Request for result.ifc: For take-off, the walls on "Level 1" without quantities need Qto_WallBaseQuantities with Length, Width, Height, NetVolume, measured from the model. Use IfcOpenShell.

First a look at what the model holds.

```python
import ifcopenshell
import ifcopenshell.util.element
import ifcopenshell.util.unit

model = ifcopenshell.open("result.ifc")
print(model.schema)
for unit_type in ("LENGTHUNIT", "AREAUNIT", "VOLUMEUNIT"):
    print(unit_type, ifcopenshell.util.unit.calculate_unit_scale(model, unit_type))
storey = next(s for s in model.by_type("IfcBuildingStorey") if s.Name == "Level 1")
walls = [e for e in ifcopenshell.util.element.get_decomposition(storey) if e.is_a("IfcWall")]
for e in sorted(walls, key=lambda e: e.id()):
    print(e.id(), e.is_a(), e.Name, list(ifcopenshell.util.element.get_psets(e, qtos_only=True)), sep=" | ")
```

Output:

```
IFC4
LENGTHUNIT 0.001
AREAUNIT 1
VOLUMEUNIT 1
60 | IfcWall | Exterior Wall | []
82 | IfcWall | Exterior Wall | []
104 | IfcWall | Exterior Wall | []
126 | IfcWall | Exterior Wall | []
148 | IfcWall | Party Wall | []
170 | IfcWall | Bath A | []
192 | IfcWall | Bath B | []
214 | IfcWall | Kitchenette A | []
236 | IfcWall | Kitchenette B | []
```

```python
import ifcopenshell
import ifcopenshell.api.pset
import ifcopenshell.geom
import ifcopenshell.util.element
import ifcopenshell.util.shape
import ifcopenshell.util.unit

model = ifcopenshell.open("result.ifc")
unit_scale = ifcopenshell.util.unit.calculate_unit_scale(model)
volume_scale = ifcopenshell.util.unit.calculate_unit_scale(model, "VOLUMEUNIT")
settings = ifcopenshell.geom.settings()

storey = next(s for s in model.by_type("IfcBuildingStorey") if s.Name == "Level 1")
walls = [e for e in ifcopenshell.util.element.get_decomposition(storey) if e.is_a("IfcWall")]

for e in sorted(walls, key=lambda e: e.id()):
    if ifcopenshell.util.element.get_psets(e, qtos_only=True, should_inherit=False):
        continue
    # Geometry comes back in metres, in the element's own axes.
    shape = ifcopenshell.geom.create_shape(settings, e)
    values = {
        "Length": ifcopenshell.util.shape.get_x(shape.geometry) / unit_scale,
        "Width": ifcopenshell.util.shape.get_y(shape.geometry) / unit_scale,
        "Height": ifcopenshell.util.shape.get_z(shape.geometry) / unit_scale,
        "NetVolume": ifcopenshell.util.shape.get_volume(shape.geometry) / volume_scale,
    }
    qto = ifcopenshell.api.pset.add_qto(model, product=e, name="Qto_WallBaseQuantities")
    ifcopenshell.api.pset.edit_qto(model, qto=qto, properties=values)
    print(e.id(), {k: round(v, 3) for k, v in values.items()})

model.write("result-out.ifc")
```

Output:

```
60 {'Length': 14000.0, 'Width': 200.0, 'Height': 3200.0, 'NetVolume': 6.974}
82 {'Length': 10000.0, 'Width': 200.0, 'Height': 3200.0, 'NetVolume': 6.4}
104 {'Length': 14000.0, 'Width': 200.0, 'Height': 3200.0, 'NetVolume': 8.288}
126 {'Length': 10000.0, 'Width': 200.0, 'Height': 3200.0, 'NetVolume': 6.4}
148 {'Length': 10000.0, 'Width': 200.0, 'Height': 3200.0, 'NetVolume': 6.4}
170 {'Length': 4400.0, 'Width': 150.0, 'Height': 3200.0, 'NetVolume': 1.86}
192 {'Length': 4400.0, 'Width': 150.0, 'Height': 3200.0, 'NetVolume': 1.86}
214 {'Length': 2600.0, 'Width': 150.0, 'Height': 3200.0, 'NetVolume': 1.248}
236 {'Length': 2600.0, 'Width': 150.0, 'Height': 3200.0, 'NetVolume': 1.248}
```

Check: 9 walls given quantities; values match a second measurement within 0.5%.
